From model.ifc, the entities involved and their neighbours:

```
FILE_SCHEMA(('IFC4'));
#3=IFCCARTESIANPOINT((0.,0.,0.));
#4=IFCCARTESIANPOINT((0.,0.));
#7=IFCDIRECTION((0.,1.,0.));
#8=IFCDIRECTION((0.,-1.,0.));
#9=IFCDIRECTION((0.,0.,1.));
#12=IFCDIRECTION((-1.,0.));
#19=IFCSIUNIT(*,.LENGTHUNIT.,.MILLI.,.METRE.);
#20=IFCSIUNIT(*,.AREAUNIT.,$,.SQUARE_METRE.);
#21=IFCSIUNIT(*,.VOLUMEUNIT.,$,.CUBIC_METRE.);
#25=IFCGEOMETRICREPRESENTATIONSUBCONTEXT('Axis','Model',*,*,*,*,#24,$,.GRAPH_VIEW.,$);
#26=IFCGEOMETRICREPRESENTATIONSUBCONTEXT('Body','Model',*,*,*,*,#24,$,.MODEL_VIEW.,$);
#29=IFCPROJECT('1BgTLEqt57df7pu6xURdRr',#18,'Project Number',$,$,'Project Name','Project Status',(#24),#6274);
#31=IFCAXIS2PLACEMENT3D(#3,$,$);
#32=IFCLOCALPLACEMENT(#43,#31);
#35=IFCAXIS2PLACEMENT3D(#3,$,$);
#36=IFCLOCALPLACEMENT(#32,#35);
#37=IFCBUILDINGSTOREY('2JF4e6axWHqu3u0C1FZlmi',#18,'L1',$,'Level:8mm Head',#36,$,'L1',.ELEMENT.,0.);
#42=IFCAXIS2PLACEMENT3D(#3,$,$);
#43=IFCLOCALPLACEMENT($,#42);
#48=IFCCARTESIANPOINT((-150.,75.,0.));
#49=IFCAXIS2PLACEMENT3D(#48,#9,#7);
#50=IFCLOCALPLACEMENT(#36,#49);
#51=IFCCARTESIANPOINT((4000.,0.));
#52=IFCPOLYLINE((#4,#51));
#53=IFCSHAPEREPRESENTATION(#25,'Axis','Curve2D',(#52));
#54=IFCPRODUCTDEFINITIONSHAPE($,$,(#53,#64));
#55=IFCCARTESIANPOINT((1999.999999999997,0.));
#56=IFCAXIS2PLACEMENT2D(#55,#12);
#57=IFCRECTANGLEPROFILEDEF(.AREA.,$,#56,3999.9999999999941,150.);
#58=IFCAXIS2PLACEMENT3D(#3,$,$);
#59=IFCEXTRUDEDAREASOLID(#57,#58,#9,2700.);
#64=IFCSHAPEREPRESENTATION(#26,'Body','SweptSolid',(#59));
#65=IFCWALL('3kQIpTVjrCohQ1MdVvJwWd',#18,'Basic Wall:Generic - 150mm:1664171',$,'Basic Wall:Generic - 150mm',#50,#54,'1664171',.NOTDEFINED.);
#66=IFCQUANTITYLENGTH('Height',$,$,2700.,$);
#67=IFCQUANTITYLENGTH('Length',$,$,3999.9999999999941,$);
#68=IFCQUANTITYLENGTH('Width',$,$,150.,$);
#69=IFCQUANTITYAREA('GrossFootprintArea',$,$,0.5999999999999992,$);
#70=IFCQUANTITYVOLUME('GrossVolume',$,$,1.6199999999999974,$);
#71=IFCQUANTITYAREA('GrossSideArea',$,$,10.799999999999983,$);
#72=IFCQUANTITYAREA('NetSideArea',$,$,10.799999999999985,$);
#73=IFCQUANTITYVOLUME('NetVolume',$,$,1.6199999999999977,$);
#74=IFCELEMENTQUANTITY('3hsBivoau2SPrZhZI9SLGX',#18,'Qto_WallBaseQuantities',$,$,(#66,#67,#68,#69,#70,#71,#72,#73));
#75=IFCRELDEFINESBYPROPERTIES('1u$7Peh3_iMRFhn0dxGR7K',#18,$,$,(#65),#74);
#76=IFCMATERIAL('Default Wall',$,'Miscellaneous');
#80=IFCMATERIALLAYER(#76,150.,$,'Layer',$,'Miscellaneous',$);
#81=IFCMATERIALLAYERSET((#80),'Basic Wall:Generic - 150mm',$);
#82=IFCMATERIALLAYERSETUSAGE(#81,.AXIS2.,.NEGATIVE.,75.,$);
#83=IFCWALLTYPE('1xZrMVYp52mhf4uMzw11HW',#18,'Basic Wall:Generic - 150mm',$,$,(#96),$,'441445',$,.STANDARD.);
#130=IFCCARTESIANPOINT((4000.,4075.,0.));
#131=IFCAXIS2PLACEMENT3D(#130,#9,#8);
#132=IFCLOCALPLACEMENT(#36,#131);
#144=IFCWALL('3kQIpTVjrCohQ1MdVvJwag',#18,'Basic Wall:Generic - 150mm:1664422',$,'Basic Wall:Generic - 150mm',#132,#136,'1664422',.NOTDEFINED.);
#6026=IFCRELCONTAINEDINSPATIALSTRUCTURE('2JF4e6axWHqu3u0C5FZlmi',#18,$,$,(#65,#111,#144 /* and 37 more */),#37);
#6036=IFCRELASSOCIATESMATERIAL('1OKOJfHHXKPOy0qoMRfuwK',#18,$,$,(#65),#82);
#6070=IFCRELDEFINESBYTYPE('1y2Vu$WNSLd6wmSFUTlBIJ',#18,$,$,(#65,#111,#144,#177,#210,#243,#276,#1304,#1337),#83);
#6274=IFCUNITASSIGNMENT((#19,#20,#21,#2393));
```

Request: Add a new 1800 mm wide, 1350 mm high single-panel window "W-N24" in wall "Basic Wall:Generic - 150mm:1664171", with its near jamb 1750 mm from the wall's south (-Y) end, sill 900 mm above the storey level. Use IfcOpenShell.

```python
import numpy as np
import ifcopenshell
import ifcopenshell.api.feature
import ifcopenshell.api.geometry
import ifcopenshell.api.pset
import ifcopenshell.api.root
import ifcopenshell.api.spatial
import ifcopenshell.geom
import ifcopenshell.util.element
import ifcopenshell.util.placement
import ifcopenshell.util.representation
import ifcopenshell.util.shape
import ifcopenshell.util.unit

model = ifcopenshell.open("model.ifc")
unit_scale = ifcopenshell.util.unit.calculate_unit_scale(model)
area_scale = ifcopenshell.util.unit.calculate_unit_scale(model, "AREAUNIT")
volume_scale = ifcopenshell.util.unit.calculate_unit_scale(model, "VOLUMEUNIT")
settings = ifcopenshell.geom.settings()


def volume(element):
    """Net volume in cubic metres, openings subtracted."""
    shape = ifcopenshell.geom.create_shape(settings, element)
    return ifcopenshell.util.shape.get_volume(shape.geometry)


wall = model.by_guid("3kQIpTVjrCohQ1MdVvJwWd")
storey = ifcopenshell.util.element.get_container(wall, ifc_class="IfcBuildingStorey")
context = ifcopenshell.util.representation.get_context(model, "Model", "Body", "MODEL_VIEW")
before = volume(wall)

width, height, from_end, sill = 1.8, 1.35, 1.75, 0.9  # metres

# The wall runs along its own X axis, and the end named is its -X end.
wall_shape = ifcopenshell.geom.create_shape(settings, wall)
x, y, z = ifcopenshell.util.shape.get_vertices(wall_shape.geometry).T
start = x.min() + from_end
face, thickness = float(y.min()), float(y.max() - y.min())
wall_matrix = ifcopenshell.util.placement.get_local_placement(wall.ObjectPlacement)
level = ifcopenshell.util.placement.get_local_placement(storey.ObjectPlacement)[2, 3]


def in_wall(x, y):
    """Placement at x, y metres in the wall's axes, at sill height."""
    matrix = wall_matrix.copy()
    matrix[:, 3] = wall_matrix @ np.array([x / unit_scale, y / unit_scale, 0.0, 1.0])
    matrix[2, 3] = level + sill / unit_scale
    return matrix


# Opening: a box that overshoots both wall faces by 50 mm.
opening = ifcopenshell.api.root.create_entity(model, ifc_class="IfcOpeningElement", predefined_type="OPENING")
box = ifcopenshell.api.geometry.add_wall_representation(
    model, context=context, length=width, height=height, thickness=thickness + 0.1
)
ifcopenshell.api.geometry.assign_representation(model, product=opening, representation=box)
ifcopenshell.api.geometry.edit_object_placement(model, product=opening, matrix=in_wall(start, face - 0.05), is_si=False)
ifcopenshell.api.feature.add_feature(model, feature=opening, element=wall)

window = ifcopenshell.api.root.create_entity(model, ifc_class="IfcWindow", name="W-N24", predefined_type="WINDOW")
window.OverallWidth, window.OverallHeight = width / unit_scale, height / unit_scale
window.PartitioningType = "SINGLE_PANEL"
body = ifcopenshell.api.geometry.add_window_representation(
    model,
    context=context,
    overall_width=window.OverallWidth,
    overall_height=window.OverallHeight,
    partition_type="SINGLE_PANEL",
)
ifcopenshell.api.geometry.assign_representation(model, product=window, representation=body)
ifcopenshell.api.spatial.assign_container(model, products=[window], relating_structure=storey)
ifcopenshell.api.feature.add_filling(model, opening=opening, element=window)

# Centre the window in the wall's thickness.
ifcopenshell.api.geometry.edit_object_placement(model, product=window, matrix=in_wall(start, face), is_si=False)
window_shape = ifcopenshell.geom.create_shape(settings, window)
depth = ifcopenshell.util.shape.get_vertices(window_shape.geometry)[:, 1]
offset = face + thickness / 2 - (depth.min() + depth.max()) / 2
ifcopenshell.api.geometry.edit_object_placement(model, product=window, matrix=in_wall(start, offset), is_si=False)

after = volume(wall)

# Update the wall's stored quantities.
qto = model.by_id(ifcopenshell.util.element.get_pset(wall, "Qto_WallBaseQuantities", should_inherit=False)["id"])
ifcopenshell.api.pset.edit_qto(model, qto=qto, properties={
    "NetSideArea": after / thickness / area_scale,
    "NetVolume": after / volume_scale,
})

print(f"wall volume {before:.3f} -> {after:.3f} m3")

model.write("model-out.ifc")
```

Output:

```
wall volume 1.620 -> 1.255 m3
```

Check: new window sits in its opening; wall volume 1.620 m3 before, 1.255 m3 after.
